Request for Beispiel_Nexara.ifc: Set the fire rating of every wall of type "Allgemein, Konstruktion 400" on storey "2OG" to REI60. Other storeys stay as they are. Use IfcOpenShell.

First a look at what the model holds.

```python
import ifcopenshell
import ifcopenshell.util.element

model = ifcopenshell.open("Beispiel_Nexara.ifc")
print(model.schema)
storey = next(s for s in model.by_type("IfcBuildingStorey") if s.Name == "2OG")
walls = [e for e in ifcopenshell.util.element.get_decomposition(storey) if e.is_a("IfcWall")]
seen = {}
for e in walls:
    element_type = ifcopenshell.util.element.get_type(e)
    key = (element_type.Name if element_type != e and element_type else None, ifcopenshell.util.element.get_pset(e, "Pset_WallCommon", "FireRating"))
    seen[key] = seen.get(key, 0) + 1
for (name, value), count in sorted(seen.items(), key=str):
    print(count, "x", name, "|", value)
```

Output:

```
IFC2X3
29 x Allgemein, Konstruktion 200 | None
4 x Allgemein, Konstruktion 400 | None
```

```python
import ifcopenshell
import ifcopenshell.api.pset
import ifcopenshell.util.element

model = ifcopenshell.open("Beispiel_Nexara.ifc")

storey = next(s for s in model.by_type("IfcBuildingStorey") if s.Name == "2OG")
walls = [e for e in ifcopenshell.util.element.get_decomposition(storey) if e.is_a("IfcWall")]

count = 0
for e in walls:
    element_type = ifcopenshell.util.element.get_type(e)
    if element_type in (None, e) or element_type.Name != "Allgemein, Konstruktion 400":
        continue
    # add_pset returns the element's existing set when there is one.
    pset = ifcopenshell.api.pset.add_pset(model, product=e, name="Pset_WallCommon")
    ifcopenshell.api.pset.edit_pset(model, pset=pset, properties={"FireRating": "REI60"})
    count += 1

print(count, "walls updated")

model.write("Beispiel_Nexara_updated.ifc")
```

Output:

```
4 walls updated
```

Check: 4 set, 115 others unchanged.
